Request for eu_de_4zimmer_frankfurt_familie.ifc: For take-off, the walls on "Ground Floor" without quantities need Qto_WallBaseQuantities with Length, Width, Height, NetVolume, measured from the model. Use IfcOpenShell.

First a look at what the model holds.

```python
import ifcopenshell
import ifcopenshell.util.element
import ifcopenshell.util.unit

model = ifcopenshell.open("eu_de_4zimmer_frankfurt_familie.ifc")
print(model.schema)
for unit_type in ("LENGTHUNIT", "AREAUNIT", "VOLUMEUNIT"):
    print(unit_type, ifcopenshell.util.unit.calculate_unit_scale(model, unit_type))
storey = next(s for s in model.by_type("IfcBuildingStorey") if s.Name == "Ground Floor")
walls = [e for e in ifcopenshell.util.element.get_decomposition(storey) if e.is_a("IfcWall")]
for e in sorted(walls, key=lambda e: e.id()):
    print(e.id(), e.is_a(), e.Name, list(ifcopenshell.util.element.get_psets(e, qtos_only=True)), sep=" | ")
```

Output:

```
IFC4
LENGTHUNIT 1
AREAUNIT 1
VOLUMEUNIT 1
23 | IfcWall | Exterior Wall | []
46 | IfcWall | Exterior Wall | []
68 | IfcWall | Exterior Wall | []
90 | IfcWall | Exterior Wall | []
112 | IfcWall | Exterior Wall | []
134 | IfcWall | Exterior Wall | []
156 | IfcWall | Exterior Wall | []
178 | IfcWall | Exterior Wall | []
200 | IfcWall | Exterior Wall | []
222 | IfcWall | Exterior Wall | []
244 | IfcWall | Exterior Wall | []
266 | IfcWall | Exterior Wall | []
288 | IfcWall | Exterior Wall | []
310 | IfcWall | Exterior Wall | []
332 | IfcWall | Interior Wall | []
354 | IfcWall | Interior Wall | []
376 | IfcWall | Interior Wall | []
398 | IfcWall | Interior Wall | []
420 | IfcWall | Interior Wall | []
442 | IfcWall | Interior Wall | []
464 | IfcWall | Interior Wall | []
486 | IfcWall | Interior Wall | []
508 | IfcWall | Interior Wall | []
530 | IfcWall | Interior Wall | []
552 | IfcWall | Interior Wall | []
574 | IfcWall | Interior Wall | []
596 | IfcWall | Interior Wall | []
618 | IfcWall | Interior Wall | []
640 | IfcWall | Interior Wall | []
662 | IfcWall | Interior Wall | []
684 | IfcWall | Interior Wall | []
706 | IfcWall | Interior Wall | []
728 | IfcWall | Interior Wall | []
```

```python
import ifcopenshell
import ifcopenshell.api.pset
import ifcopenshell.geom
import ifcopenshell.util.element
import ifcopenshell.util.shape
import ifcopenshell.util.unit

model = ifcopenshell.open("eu_de_4zimmer_frankfurt_familie.ifc")
unit_scale = ifcopenshell.util.unit.calculate_unit_scale(model)
volume_scale = ifcopenshell.util.unit.calculate_unit_scale(model, "VOLUMEUNIT")
settings = ifcopenshell.geom.settings()

storey = next(s for s in model.by_type("IfcBuildingStorey") if s.Name == "Ground Floor")
walls = [e for e in ifcopenshell.util.element.get_decomposition(storey) if e.is_a("IfcWall")]

for e in sorted(walls, key=lambda e: e.id()):
    if ifcopenshell.util.element.get_psets(e, qtos_only=True, should_inherit=False):
        continue
    # Geometry comes back in metres, in the element's own axes.
    shape = ifcopenshell.geom.create_shape(settings, e)
    values = {
        "Length": ifcopenshell.util.shape.get_x(shape.geometry) / unit_scale,
        "Width": ifcopenshell.util.shape.get_y(shape.geometry) / unit_scale,
        "Height": ifcopenshell.util.shape.get_z(shape.geometry) / unit_scale,
        "NetVolume": ifcopenshell.util.shape.get_volume(shape.geometry) / volume_scale,
    }
    qto = ifcopenshell.api.pset.add_qto(model, product=e, name="Qto_WallBaseQuantities")
    ifcopenshell.api.pset.edit_qto(model, qto=qto, properties=values)
    print(e.id(), {k: round(v, 3) for k, v in values.items()})

model.write("eu_de_4zimmer_frankfurt_familie_updated.ifc")
```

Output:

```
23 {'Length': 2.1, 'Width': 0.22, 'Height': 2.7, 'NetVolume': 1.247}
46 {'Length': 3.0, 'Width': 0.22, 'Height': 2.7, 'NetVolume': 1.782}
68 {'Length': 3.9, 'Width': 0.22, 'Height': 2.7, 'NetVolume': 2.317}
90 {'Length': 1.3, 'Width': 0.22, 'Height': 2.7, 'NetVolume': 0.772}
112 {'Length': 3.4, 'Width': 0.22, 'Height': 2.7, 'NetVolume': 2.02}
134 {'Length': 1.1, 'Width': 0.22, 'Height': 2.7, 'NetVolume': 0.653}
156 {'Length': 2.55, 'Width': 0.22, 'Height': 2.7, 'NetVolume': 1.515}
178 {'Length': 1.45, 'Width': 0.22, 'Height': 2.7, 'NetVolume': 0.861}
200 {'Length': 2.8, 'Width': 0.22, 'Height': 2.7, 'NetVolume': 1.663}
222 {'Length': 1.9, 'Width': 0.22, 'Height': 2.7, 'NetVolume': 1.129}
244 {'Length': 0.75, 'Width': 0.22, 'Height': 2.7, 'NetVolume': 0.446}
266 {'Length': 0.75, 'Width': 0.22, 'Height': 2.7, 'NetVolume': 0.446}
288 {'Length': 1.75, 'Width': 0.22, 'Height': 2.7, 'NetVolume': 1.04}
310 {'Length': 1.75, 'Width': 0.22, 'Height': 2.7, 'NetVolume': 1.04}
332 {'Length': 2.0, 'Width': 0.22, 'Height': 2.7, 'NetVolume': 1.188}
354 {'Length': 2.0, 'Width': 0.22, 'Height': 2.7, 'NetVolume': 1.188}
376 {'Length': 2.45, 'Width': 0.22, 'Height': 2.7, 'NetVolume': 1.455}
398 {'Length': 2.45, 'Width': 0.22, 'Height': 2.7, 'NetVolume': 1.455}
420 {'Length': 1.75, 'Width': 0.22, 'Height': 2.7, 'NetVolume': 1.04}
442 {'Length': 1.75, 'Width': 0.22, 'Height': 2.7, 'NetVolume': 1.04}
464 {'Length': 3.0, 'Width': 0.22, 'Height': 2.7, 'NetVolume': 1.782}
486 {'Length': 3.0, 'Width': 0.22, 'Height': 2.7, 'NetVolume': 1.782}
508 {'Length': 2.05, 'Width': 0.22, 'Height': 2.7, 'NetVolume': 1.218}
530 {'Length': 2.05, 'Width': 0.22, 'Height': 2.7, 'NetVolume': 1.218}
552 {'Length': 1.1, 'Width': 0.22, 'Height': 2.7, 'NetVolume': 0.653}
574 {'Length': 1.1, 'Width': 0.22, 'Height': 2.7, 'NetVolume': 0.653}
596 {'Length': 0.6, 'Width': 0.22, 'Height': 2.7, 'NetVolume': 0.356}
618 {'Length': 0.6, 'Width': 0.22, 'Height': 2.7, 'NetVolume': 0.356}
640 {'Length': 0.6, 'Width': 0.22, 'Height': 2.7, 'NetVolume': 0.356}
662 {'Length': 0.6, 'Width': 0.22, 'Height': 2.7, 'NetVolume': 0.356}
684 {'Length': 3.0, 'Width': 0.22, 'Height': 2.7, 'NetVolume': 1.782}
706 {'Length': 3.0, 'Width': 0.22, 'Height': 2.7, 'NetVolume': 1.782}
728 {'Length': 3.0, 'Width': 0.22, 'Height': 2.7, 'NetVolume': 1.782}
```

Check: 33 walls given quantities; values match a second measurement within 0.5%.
